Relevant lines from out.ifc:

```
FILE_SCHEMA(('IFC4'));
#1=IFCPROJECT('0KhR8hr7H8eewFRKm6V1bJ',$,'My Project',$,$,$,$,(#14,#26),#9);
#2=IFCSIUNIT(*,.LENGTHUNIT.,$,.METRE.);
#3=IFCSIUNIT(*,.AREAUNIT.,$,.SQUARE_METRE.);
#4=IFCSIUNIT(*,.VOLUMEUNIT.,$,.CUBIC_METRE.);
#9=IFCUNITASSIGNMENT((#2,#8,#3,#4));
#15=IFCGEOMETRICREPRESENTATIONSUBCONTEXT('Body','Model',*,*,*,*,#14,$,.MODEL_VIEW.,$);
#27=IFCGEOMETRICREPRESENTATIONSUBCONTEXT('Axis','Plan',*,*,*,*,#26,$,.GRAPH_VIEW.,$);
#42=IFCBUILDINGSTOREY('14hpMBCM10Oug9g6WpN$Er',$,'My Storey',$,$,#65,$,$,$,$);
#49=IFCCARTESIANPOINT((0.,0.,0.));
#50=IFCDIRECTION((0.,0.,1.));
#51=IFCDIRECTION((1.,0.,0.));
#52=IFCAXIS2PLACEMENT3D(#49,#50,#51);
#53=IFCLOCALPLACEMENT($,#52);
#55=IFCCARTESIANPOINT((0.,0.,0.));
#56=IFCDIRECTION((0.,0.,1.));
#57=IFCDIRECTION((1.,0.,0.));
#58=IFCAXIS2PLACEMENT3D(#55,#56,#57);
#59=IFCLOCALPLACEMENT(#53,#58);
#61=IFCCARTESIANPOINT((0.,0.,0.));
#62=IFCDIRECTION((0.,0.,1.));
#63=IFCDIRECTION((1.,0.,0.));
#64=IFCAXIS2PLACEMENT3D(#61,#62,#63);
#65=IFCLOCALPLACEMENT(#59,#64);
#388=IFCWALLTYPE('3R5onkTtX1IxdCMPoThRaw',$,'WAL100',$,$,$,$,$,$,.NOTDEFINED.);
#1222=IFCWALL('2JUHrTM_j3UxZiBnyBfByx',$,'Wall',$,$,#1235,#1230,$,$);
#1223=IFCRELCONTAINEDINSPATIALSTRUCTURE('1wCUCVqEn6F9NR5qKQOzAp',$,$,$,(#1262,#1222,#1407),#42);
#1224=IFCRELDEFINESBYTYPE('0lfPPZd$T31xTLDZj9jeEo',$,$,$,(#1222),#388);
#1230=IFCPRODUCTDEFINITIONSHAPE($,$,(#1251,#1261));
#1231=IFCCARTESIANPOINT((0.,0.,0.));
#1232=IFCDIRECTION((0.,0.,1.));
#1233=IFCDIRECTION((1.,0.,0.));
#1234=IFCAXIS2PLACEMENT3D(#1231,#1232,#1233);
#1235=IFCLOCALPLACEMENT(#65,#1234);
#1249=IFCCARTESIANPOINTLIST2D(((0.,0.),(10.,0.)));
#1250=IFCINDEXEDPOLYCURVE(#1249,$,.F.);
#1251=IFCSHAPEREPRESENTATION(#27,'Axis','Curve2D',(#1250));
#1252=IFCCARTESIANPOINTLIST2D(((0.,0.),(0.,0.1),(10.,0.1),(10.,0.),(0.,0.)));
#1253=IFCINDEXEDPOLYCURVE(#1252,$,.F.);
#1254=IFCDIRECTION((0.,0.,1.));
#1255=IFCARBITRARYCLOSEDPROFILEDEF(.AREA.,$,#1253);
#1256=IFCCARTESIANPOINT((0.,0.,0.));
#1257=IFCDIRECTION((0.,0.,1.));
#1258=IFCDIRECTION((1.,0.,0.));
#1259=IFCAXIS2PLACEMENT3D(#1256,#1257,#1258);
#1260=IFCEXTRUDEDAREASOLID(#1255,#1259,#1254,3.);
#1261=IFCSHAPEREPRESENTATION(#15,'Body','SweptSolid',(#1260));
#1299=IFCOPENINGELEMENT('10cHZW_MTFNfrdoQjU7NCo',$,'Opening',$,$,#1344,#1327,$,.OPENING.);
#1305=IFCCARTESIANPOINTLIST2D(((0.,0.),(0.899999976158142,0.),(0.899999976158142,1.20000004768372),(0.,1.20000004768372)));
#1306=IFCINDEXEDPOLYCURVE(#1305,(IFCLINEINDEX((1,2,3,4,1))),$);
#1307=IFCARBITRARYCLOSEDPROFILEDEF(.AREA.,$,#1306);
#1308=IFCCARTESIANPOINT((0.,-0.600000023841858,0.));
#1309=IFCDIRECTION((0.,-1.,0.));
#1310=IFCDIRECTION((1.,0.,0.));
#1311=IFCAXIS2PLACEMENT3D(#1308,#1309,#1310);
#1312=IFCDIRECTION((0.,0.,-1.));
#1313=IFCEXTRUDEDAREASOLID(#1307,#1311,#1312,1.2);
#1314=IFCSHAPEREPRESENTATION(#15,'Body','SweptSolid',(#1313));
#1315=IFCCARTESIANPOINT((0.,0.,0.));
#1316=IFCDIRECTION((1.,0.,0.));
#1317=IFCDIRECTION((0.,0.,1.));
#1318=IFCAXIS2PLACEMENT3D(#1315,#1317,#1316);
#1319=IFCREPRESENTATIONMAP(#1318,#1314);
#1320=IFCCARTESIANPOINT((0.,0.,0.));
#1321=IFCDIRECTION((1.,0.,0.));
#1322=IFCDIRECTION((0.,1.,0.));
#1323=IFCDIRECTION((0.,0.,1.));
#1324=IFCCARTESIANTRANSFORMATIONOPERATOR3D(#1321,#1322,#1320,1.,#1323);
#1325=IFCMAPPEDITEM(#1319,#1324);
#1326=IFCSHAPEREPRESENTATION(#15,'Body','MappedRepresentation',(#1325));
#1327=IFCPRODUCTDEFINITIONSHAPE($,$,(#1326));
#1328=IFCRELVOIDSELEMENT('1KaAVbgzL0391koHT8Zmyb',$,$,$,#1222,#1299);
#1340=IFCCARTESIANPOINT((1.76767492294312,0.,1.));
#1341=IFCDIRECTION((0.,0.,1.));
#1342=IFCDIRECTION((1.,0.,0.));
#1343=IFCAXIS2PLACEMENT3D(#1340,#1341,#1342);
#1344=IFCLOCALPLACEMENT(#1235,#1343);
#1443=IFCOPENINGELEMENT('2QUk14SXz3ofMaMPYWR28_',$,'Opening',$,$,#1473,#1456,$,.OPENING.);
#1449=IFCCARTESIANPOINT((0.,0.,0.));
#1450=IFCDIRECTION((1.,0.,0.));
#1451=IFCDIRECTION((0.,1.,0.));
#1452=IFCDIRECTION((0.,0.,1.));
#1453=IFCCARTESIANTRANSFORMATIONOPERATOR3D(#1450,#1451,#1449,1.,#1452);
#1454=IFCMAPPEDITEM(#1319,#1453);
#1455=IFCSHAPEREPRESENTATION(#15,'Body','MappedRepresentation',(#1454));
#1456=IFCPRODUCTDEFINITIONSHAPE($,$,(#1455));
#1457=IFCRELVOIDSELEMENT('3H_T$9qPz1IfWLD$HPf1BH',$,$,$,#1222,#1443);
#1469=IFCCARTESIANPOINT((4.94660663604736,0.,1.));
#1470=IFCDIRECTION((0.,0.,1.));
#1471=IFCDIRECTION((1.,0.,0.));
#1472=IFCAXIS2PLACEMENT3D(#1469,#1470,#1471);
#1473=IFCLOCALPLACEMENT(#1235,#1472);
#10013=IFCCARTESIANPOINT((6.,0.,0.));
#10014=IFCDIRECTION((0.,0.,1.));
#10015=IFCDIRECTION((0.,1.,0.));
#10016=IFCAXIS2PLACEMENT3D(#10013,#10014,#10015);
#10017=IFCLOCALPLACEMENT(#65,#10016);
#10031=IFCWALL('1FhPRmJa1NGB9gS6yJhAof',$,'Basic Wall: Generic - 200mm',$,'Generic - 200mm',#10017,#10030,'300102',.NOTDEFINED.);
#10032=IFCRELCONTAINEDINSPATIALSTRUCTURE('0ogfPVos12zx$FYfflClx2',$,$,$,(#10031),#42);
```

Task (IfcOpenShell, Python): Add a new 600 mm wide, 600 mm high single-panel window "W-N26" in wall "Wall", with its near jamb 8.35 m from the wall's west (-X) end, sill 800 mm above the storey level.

```python
import numpy as np
import ifcopenshell
import ifcopenshell.api.feature
import ifcopenshell.api.geometry
import ifcopenshell.api.root
import ifcopenshell.api.spatial
import ifcopenshell.geom
import ifcopenshell.util.element
import ifcopenshell.util.placement
import ifcopenshell.util.representation
import ifcopenshell.util.shape
import ifcopenshell.util.unit

model = ifcopenshell.open("out.ifc")
unit_scale = ifcopenshell.util.unit.calculate_unit_scale(model)
settings = ifcopenshell.geom.settings()


def volume(element):
    """Net volume in cubic metres, openings subtracted."""
    shape = ifcopenshell.geom.create_shape(settings, element)
    return ifcopenshell.util.shape.get_volume(shape.geometry)


wall = model.by_guid("2JUHrTM_j3UxZiBnyBfByx")
storey = ifcopenshell.util.element.get_container(wall, ifc_class="IfcBuildingStorey")
context = ifcopenshell.util.representation.get_context(model, "Model", "Body", "MODEL_VIEW")
before = volume(wall)

width, height, from_end, sill = 0.6, 0.6, 8.35, 0.8  # metres

# The wall runs along its own X axis, and the end named is its -X end.
wall_shape = ifcopenshell.geom.create_shape(settings, wall)
x, y, z = ifcopenshell.util.shape.get_vertices(wall_shape.geometry).T
start = x.min() + from_end
face, thickness = float(y.min()), float(y.max() - y.min())
wall_matrix = ifcopenshell.util.placement.get_local_placement(wall.ObjectPlacement)
level = ifcopenshell.util.placement.get_local_placement(storey.ObjectPlacement)[2, 3]


def in_wall(x, y):
    """Placement at x, y metres in the wall's axes, at sill height."""
    matrix = wall_matrix.copy()
    matrix[:, 3] = wall_matrix @ np.array([x / unit_scale, y / unit_scale, 0.0, 1.0])
    matrix[2, 3] = level + sill / unit_scale
    return matrix


# Opening: a box that overshoots both wall faces by 50 mm.
opening = ifcopenshell.api.root.create_entity(model, ifc_class="IfcOpeningElement", predefined_type="OPENING")
box = ifcopenshell.api.geometry.add_wall_representation(
    model, context=context, length=width, height=height, thickness=thickness + 0.1
)
ifcopenshell.api.geometry.assign_representation(model, product=opening, representation=box)
ifcopenshell.api.geometry.edit_object_placement(model, product=opening, matrix=in_wall(start, face - 0.05), is_si=False)
ifcopenshell.api.feature.add_feature(model, feature=opening, element=wall)

window = ifcopenshell.api.root.create_entity(model, ifc_class="IfcWindow", name="W-N26", predefined_type="WINDOW")
window.OverallWidth, window.OverallHeight = width / unit_scale, height / unit_scale
window.PartitioningType = "SINGLE_PANEL"
body = ifcopenshell.api.geometry.add_window_representation(
    model,
    context=context,
    overall_width=window.OverallWidth,
    overall_height=window.OverallHeight,
    partition_type="SINGLE_PANEL",
)
ifcopenshell.api.geometry.assign_representation(model, product=window, representation=body)
ifcopenshell.api.spatial.assign_container(model, products=[window], relating_structure=storey)
ifcopenshell.api.feature.add_filling(model, opening=opening, element=window)

# Centre the window in the wall's thickness.
ifcopenshell.api.geometry.edit_object_placement(model, product=window, matrix=in_wall(start, face), is_si=False)
window_shape = ifcopenshell.geom.create_shape(settings, window)
depth = ifcopenshell.util.shape.get_vertices(window_shape.geometry)[:, 1]
offset = face + thickness / 2 - (depth.min() + depth.max()) / 2
ifcopenshell.api.geometry.edit_object_placement(model, product=window, matrix=in_wall(start, offset), is_si=False)

after = volume(wall)

print(f"wall volume {before:.3f} -> {after:.3f} m3")

model.write("out_edited.ifc")
```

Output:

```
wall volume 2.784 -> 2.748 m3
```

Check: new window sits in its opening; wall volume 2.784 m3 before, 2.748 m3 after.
